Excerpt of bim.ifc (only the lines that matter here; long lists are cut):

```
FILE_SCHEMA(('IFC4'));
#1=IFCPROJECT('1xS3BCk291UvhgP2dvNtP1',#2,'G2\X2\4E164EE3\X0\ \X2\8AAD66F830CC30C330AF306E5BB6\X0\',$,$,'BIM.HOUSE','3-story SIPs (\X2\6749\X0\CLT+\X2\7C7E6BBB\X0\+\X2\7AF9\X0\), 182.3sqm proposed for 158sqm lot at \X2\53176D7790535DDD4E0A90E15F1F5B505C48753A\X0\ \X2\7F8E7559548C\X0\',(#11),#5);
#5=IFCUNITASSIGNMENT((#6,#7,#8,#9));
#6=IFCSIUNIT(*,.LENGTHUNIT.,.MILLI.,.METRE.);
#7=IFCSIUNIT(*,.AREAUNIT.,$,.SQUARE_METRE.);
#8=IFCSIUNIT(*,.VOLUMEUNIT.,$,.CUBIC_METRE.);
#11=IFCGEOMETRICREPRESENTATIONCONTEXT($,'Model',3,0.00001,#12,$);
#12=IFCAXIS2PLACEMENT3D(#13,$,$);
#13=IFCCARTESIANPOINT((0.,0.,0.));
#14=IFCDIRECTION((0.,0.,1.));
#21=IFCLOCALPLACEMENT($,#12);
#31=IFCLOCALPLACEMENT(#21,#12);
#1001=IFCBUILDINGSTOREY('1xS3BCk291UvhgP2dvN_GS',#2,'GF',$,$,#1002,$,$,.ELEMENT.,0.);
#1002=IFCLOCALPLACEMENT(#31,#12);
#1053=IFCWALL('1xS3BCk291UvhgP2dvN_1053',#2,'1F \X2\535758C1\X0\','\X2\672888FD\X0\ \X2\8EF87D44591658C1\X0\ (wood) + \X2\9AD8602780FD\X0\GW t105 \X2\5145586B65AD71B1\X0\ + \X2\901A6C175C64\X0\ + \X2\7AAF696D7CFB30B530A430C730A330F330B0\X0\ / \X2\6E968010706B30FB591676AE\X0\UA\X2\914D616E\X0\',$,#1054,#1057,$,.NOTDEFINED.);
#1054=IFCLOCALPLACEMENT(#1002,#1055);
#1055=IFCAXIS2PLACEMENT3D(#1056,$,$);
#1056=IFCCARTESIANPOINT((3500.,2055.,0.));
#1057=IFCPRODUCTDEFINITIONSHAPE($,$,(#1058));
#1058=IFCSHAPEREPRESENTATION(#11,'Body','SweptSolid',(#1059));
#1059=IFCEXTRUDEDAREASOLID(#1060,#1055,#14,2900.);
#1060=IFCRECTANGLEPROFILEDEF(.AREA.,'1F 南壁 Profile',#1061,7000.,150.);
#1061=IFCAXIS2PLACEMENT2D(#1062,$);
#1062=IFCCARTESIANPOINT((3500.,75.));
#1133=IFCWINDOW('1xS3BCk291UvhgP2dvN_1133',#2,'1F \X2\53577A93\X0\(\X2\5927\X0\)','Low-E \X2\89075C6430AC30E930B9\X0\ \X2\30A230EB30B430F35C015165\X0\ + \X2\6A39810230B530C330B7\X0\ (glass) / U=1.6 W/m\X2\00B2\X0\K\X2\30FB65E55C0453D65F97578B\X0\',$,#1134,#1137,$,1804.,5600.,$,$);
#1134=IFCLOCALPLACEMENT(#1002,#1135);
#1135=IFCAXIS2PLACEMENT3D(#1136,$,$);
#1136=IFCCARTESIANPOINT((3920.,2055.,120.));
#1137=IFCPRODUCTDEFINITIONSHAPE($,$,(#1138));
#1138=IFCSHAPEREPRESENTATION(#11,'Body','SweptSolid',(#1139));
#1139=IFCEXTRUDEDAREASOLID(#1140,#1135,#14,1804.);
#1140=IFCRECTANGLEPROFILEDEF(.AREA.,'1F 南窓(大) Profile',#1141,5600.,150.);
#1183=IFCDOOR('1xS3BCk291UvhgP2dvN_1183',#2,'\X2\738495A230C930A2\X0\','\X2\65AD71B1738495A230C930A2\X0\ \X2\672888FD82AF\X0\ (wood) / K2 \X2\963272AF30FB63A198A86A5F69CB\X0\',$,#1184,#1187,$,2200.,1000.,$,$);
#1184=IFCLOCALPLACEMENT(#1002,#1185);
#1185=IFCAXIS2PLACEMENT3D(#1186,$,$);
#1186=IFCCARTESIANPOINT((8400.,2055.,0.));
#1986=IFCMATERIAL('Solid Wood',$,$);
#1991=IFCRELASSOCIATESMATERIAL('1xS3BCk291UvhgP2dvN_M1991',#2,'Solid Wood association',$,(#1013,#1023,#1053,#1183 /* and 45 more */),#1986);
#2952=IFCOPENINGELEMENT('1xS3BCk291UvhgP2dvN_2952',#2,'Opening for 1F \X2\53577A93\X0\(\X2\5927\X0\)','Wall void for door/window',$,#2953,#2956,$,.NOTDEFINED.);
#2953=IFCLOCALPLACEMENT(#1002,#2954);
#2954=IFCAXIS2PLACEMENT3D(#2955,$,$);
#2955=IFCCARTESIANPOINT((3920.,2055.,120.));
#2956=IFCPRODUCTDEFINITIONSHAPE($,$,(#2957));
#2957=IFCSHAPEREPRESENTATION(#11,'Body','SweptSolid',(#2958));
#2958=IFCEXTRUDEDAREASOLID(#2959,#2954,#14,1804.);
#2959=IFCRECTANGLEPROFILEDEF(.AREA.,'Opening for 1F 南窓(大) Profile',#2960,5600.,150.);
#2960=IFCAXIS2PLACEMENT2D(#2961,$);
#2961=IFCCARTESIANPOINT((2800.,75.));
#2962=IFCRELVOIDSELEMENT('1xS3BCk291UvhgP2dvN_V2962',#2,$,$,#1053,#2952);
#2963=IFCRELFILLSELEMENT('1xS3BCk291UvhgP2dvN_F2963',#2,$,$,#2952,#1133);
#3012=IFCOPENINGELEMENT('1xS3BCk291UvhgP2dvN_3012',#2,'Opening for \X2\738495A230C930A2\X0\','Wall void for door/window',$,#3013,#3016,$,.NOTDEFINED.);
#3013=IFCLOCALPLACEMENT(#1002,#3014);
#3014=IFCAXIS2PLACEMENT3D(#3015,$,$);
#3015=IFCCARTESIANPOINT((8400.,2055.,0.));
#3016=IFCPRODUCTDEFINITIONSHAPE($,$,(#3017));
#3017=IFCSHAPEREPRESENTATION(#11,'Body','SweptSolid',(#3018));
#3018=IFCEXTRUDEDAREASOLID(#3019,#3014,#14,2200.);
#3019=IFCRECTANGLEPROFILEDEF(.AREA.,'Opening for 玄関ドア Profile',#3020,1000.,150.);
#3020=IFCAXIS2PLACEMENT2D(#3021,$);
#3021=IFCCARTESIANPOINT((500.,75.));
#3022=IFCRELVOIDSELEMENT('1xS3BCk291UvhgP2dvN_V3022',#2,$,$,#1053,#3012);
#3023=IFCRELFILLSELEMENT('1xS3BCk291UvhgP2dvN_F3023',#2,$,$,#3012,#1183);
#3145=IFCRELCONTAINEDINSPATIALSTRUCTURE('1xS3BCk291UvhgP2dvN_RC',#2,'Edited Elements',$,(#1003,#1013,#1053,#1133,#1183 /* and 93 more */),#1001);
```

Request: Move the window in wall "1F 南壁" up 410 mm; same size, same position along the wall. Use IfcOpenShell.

```python
import numpy as np
import ifcopenshell
import ifcopenshell.api.geometry
import ifcopenshell.util.placement
import ifcopenshell.util.unit

model = ifcopenshell.open("bim.ifc")
unit_scale = ifcopenshell.util.unit.calculate_unit_scale(model)

window = model.by_id(1133)
opening = window.FillsVoids[0].RelatingOpeningElement
dz = 0.41 / unit_scale

shift = np.array([0.0, 0.0, dz])
# The window is not placed relative to its opening, so move both.
for product in (opening, window):
    matrix = ifcopenshell.util.placement.get_local_placement(product.ObjectPlacement)
    matrix[:3, 3] += shift
    ifcopenshell.api.geometry.edit_object_placement(model, product=product, matrix=matrix, is_si=False)

print(f"moved by {dz * unit_scale:+.3f} m")

model.write("bim_edited.ifc")
```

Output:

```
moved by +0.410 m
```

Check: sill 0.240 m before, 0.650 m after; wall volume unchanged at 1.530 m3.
